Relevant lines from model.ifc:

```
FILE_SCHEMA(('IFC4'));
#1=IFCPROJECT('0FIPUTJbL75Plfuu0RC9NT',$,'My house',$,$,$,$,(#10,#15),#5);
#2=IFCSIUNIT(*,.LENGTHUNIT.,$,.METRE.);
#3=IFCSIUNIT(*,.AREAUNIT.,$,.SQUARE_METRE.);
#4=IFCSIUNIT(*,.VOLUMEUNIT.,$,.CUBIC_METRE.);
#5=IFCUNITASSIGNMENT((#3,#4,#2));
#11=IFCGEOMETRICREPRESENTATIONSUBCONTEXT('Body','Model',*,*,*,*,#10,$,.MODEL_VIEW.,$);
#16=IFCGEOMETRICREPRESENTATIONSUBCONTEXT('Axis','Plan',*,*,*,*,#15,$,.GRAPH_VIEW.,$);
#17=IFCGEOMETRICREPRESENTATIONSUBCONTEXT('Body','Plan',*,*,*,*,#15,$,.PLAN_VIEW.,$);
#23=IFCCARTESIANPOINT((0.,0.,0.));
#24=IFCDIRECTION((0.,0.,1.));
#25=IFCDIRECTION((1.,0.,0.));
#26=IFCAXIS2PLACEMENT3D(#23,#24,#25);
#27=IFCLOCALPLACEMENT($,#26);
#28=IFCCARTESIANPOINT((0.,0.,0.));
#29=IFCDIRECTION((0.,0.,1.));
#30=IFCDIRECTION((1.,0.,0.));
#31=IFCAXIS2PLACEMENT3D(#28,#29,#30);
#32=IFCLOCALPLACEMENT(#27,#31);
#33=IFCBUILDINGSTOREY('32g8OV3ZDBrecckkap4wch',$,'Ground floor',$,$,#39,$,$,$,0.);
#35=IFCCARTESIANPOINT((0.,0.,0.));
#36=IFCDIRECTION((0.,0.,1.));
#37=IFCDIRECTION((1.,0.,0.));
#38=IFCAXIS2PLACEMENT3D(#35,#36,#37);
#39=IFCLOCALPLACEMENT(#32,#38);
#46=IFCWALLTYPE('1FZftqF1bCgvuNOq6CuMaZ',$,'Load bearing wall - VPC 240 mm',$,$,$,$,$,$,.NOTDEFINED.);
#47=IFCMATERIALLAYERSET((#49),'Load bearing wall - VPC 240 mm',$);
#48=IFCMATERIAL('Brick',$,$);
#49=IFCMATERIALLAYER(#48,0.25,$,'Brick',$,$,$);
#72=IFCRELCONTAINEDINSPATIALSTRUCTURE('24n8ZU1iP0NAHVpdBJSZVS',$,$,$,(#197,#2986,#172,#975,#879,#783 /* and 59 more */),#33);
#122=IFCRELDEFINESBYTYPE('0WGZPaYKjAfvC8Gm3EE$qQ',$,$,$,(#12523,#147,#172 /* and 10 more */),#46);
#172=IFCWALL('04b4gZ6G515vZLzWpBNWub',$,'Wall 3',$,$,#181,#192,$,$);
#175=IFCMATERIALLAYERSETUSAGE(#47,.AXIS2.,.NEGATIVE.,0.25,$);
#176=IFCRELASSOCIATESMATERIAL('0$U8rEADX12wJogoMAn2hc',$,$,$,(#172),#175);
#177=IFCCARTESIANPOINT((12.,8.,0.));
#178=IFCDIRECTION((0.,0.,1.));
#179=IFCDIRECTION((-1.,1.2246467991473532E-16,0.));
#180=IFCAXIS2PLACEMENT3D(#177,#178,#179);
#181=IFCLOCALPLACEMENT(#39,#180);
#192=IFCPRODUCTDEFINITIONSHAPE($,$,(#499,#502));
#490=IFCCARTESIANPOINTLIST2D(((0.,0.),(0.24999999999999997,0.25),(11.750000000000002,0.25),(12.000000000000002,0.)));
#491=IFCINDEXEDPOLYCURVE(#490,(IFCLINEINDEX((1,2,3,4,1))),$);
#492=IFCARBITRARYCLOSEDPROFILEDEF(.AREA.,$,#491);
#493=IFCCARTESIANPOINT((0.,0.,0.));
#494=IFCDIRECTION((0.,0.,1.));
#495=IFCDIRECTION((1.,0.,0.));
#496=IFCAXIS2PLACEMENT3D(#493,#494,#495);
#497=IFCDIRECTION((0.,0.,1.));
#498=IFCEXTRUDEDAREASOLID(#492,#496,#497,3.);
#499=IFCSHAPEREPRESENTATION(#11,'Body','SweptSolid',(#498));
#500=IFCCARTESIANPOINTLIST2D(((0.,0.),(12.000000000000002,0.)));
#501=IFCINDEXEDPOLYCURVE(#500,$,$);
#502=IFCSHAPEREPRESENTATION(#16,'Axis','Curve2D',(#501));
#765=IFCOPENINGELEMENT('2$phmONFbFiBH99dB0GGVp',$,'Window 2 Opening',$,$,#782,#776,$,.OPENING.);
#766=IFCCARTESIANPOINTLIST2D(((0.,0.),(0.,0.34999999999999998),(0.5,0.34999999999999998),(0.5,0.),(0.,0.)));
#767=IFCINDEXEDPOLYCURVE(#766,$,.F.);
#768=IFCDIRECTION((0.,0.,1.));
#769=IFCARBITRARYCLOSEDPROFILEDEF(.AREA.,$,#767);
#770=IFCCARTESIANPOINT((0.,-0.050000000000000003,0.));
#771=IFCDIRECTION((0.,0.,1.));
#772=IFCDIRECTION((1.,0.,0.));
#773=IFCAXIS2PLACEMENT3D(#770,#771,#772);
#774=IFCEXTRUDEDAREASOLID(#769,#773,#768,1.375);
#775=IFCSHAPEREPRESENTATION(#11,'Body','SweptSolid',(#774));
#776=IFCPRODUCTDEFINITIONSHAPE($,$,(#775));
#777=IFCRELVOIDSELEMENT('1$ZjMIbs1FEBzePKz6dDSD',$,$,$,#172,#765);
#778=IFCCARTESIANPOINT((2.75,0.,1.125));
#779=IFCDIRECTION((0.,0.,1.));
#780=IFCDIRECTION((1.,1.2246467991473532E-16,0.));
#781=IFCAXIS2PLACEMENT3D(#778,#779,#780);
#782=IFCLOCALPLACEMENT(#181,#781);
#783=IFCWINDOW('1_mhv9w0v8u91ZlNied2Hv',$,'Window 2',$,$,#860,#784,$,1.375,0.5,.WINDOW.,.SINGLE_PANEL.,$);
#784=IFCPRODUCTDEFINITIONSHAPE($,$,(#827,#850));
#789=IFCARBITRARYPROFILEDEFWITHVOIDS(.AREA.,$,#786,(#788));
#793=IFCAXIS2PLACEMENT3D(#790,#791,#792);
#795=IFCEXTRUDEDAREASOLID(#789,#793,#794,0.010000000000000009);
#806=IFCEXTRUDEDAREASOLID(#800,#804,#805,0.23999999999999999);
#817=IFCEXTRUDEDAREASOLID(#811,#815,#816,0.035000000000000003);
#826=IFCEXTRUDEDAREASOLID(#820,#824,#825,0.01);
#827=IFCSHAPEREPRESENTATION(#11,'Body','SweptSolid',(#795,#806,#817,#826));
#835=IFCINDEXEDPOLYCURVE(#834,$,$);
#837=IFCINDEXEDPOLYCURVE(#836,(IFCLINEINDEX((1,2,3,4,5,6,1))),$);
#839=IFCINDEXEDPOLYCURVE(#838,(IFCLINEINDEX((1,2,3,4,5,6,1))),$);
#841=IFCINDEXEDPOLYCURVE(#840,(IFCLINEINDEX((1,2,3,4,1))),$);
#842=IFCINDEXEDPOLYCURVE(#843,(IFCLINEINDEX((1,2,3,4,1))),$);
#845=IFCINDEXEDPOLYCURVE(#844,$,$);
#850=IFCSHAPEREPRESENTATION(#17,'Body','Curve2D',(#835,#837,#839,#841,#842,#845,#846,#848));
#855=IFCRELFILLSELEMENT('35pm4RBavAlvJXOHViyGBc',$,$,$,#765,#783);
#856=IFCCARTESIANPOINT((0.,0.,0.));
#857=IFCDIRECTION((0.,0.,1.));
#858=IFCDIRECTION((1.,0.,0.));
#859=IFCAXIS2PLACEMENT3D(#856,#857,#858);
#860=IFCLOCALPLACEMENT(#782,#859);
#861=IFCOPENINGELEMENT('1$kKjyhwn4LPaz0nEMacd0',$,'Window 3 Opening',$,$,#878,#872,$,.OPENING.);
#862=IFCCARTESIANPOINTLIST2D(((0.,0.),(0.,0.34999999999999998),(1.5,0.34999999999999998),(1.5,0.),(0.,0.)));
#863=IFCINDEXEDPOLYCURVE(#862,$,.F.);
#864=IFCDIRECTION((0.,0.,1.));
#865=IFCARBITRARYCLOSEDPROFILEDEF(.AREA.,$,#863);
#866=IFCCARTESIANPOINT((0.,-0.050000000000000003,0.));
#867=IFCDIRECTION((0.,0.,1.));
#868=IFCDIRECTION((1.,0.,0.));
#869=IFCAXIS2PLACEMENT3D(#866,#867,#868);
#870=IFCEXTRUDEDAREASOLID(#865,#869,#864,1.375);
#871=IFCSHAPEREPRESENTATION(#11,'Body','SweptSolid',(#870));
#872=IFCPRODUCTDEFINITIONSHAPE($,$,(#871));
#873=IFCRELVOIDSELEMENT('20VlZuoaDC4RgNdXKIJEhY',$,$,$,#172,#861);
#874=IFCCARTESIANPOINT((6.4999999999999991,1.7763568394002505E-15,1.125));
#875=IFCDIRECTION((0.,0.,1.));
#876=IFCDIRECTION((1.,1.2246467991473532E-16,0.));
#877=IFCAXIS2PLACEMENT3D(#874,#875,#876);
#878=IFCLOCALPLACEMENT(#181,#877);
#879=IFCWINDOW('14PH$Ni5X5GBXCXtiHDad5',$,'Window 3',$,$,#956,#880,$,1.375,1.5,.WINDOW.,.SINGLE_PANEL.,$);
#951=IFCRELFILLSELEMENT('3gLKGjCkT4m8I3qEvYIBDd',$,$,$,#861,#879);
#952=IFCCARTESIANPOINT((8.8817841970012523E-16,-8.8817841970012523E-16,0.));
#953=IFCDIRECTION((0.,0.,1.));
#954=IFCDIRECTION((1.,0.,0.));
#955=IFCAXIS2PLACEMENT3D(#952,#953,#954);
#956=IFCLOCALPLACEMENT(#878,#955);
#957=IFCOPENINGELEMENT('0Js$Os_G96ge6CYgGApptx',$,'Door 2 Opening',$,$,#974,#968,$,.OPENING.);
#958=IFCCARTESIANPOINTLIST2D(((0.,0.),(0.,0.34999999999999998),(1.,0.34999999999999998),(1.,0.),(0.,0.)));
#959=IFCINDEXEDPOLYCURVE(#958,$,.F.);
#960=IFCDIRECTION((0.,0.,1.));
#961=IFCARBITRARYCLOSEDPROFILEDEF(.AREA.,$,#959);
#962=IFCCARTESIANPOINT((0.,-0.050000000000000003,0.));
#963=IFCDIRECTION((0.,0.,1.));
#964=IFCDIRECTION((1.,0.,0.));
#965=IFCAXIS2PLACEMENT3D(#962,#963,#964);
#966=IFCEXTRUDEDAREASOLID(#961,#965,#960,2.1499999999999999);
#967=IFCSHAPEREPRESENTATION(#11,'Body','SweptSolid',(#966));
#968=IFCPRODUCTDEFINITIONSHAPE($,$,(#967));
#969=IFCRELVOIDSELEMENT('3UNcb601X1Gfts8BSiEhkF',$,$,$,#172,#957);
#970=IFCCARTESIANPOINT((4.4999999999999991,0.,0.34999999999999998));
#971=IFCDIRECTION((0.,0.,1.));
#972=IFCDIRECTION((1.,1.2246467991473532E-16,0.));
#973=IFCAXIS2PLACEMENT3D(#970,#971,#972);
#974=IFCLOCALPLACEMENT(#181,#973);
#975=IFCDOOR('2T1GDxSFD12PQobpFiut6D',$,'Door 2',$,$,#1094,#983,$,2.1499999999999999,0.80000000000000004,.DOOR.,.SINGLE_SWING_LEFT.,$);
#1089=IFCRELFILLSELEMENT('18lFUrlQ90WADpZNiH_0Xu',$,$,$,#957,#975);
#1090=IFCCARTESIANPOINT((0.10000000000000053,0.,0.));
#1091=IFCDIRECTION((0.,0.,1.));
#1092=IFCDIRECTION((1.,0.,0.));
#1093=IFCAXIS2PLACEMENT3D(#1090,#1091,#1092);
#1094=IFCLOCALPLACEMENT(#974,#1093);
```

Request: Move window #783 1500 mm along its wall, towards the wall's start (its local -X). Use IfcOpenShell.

```python
import ifcopenshell
import ifcopenshell.api.geometry
import ifcopenshell.util.placement

model = ifcopenshell.open("model.ifc")

window = model.by_guid("1_mhv9w0v8u91ZlNied2Hv")
opening = window.FillsVoids[0].RelatingOpeningElement
wall = opening.VoidsElements[0].RelatingBuildingElement

wall_matrix = ifcopenshell.util.placement.get_local_placement(wall.ObjectPlacement)
shift = wall_matrix[:3, 0] * -1.5
before = ifcopenshell.util.placement.get_local_placement(window.ObjectPlacement)[:3, 3].copy()

# The window is placed relative to its opening, so it follows when the opening moves.
matrix = ifcopenshell.util.placement.get_local_placement(opening.ObjectPlacement)
matrix[:3, 3] += shift
ifcopenshell.api.geometry.edit_object_placement(
    model, product=opening, matrix=matrix, is_si=False, should_transform_children=True
)

after = ifcopenshell.util.placement.get_local_placement(window.ObjectPlacement)[:3, 3]
print("window moved by", (after - before).round(3) + 0.0)

model.write("model-out.ifc")
```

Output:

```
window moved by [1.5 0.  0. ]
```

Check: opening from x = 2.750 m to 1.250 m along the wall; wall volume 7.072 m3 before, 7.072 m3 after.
